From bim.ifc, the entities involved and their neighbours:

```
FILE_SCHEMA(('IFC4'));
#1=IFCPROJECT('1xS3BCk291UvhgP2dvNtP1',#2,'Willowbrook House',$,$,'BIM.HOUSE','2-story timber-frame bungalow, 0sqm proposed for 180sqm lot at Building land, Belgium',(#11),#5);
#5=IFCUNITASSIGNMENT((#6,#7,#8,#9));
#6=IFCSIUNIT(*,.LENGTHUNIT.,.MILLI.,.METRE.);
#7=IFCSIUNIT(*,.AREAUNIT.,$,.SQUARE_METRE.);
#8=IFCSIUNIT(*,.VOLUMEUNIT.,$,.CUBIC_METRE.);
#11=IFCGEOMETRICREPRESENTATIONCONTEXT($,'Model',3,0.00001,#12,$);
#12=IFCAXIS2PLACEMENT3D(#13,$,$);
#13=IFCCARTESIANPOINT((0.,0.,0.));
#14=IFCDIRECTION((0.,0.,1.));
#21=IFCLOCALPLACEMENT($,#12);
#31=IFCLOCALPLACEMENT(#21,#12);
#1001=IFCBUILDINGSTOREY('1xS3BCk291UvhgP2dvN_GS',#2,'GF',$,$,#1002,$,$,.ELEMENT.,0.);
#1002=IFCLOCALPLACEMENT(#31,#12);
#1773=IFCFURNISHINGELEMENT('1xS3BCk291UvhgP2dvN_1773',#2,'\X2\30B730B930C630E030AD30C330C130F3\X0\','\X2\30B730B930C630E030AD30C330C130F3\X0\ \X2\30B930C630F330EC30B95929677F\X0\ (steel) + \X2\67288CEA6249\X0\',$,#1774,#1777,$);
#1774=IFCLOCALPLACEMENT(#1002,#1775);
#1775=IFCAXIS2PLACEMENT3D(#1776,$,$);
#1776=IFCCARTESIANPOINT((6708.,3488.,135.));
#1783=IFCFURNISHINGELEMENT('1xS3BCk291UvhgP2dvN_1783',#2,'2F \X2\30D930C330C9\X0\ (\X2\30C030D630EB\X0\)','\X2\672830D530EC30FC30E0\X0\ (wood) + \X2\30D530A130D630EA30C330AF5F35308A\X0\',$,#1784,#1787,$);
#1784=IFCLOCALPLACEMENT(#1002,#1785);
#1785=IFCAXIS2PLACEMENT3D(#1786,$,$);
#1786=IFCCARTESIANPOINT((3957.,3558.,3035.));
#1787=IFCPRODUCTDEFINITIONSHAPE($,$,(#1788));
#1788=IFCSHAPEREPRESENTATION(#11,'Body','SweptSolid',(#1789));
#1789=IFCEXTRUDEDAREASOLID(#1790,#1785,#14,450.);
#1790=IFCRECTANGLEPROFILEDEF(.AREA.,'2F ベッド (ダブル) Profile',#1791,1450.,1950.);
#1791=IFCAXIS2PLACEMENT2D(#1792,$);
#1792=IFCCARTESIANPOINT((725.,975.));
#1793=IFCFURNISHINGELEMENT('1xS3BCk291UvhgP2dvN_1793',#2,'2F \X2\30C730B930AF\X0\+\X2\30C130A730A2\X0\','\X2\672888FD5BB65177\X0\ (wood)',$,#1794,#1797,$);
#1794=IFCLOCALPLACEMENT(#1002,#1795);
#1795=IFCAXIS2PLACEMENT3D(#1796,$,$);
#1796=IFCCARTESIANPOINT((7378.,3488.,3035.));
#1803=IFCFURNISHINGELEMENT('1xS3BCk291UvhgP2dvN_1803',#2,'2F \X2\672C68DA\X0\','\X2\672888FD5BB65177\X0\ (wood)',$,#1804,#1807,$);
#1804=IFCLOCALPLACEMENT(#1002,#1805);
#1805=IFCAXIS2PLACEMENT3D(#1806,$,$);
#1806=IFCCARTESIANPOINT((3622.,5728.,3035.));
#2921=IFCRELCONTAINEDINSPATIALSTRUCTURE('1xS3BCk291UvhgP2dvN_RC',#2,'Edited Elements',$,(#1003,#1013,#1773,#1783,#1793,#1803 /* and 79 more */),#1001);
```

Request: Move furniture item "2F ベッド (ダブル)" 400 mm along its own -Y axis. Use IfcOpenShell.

```python
import ifcopenshell
import ifcopenshell.api.geometry
import ifcopenshell.util.placement

model = ifcopenshell.open("bim.ifc")

item = model.by_guid("1xS3BCk291UvhgP2dvN_1783")
matrix = ifcopenshell.util.placement.get_local_placement(item.ObjectPlacement)
matrix[:3, 3] -= matrix[:3, 1] * 400.0
ifcopenshell.api.geometry.edit_object_placement(model, product=item, matrix=matrix, is_si=False)

print(ifcopenshell.util.placement.get_local_placement(item.ObjectPlacement).round(3) + 0.0)

model.write("bim_updated.ifc")
```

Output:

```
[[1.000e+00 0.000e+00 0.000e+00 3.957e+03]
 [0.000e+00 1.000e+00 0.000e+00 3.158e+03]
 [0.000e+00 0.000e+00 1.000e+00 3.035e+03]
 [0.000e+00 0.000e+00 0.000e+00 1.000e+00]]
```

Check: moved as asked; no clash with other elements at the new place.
